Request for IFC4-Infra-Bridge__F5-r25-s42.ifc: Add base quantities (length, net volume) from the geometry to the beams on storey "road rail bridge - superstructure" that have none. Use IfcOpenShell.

First a look at what the model holds.

```python
import ifcopenshell
import ifcopenshell.util.element
import ifcopenshell.util.unit

model = ifcopenshell.open("IFC4-Infra-Bridge__F5-r25-s42.ifc")
print(model.schema)
for unit_type in ("LENGTHUNIT", "AREAUNIT", "VOLUMEUNIT"):
    print(unit_type, ifcopenshell.util.unit.calculate_unit_scale(model, unit_type))
storey = next(s for s in model.by_type("IfcBuildingStorey") if s.Name == "road rail bridge - superstructure")
beams = [e for e in ifcopenshell.util.element.get_decomposition(storey) if e.is_a("IfcBeam")]
for e in sorted(beams, key=lambda e: e.id()):
    print(e.id(), e.is_a(), e.Name, list(ifcopenshell.util.element.get_psets(e, qtos_only=True)), sep=" | ")
```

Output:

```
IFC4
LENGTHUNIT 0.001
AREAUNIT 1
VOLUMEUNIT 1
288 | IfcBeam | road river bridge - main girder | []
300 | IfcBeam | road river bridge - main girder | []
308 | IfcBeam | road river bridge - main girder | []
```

```python
import ifcopenshell
import ifcopenshell.api.pset
import ifcopenshell.geom
import ifcopenshell.util.element
import ifcopenshell.util.shape
import ifcopenshell.util.unit

model = ifcopenshell.open("IFC4-Infra-Bridge__F5-r25-s42.ifc")
unit_scale = ifcopenshell.util.unit.calculate_unit_scale(model)
volume_scale = ifcopenshell.util.unit.calculate_unit_scale(model, "VOLUMEUNIT")
settings = ifcopenshell.geom.settings()

storey = next(s for s in model.by_type("IfcBuildingStorey") if s.Name == "road rail bridge - superstructure")
beams = [e for e in ifcopenshell.util.element.get_decomposition(storey) if e.is_a("IfcBeam")]

for e in sorted(beams, key=lambda e: e.id()):
    if ifcopenshell.util.element.get_psets(e, qtos_only=True, should_inherit=False):
        continue
    # Geometry comes back in metres, in the element's own axes.
    shape = ifcopenshell.geom.create_shape(settings, e)
    values = {
        "Length": ifcopenshell.util.shape.get_max_xyz(shape.geometry) / unit_scale,
        "NetVolume": ifcopenshell.util.shape.get_volume(shape.geometry) / volume_scale,
    }
    qto = ifcopenshell.api.pset.add_qto(model, product=e, name="Qto_BeamBaseQuantities")
    ifcopenshell.api.pset.edit_qto(model, qto=qto, properties=values)
    print(e.id(), {k: round(v, 3) for k, v in values.items()})

model.write("IFC4-Infra-Bridge__F5-r25-s42-out.ifc")
```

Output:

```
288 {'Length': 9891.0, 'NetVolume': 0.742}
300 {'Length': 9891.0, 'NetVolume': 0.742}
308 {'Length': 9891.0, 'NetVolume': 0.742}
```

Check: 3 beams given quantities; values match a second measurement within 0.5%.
